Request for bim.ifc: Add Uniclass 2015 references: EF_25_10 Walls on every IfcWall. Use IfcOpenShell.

First a look at what the model holds.

```python
import ifcopenshell

model = ifcopenshell.open("bim.ifc")
print(model.schema)
print("classifications:", [c.Name for c in model.by_type("IfcClassification")])
for ifc_class in ("IfcDoor", "IfcRoof", "IfcStair", "IfcWall", "IfcWindow"):
    print(ifc_class, len(model.by_type(ifc_class)))
```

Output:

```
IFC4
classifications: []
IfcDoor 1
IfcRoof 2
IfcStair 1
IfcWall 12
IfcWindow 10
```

```python
import ifcopenshell
import ifcopenshell.api.classification

model = ifcopenshell.open("bim.ifc")

system = ifcopenshell.api.classification.add_classification(model, classification="Uniclass 2015")

codes = {
    "IfcWall": ("EF_25_10", "Walls"),
}
for ifc_class, (code, name) in codes.items():
    products = model.by_type(ifc_class)
    ifcopenshell.api.classification.add_reference(
        model, products=products, classification=system, identification=code, name=name
    )
    print(code, len(products))

model.write("bim-out.ifc")
```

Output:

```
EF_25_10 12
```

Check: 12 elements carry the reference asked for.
